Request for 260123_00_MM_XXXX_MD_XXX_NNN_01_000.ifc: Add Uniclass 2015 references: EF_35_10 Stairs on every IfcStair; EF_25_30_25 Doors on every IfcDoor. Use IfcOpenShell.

First a look at what the model holds.

```python
import ifcopenshell

model = ifcopenshell.open("260123_00_MM_XXXX_MD_XXX_NNN_01_000.ifc")
print(model.schema)
print("classifications:", [c.Name for c in model.by_type("IfcClassification")])
for ifc_class in ("IfcDoor", "IfcRoof", "IfcStair", "IfcWall", "IfcWindow"):
    print(ifc_class, len(model.by_type(ifc_class)))
```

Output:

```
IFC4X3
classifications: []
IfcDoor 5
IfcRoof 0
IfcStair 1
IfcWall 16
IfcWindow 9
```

```python
import ifcopenshell
import ifcopenshell.api.classification

model = ifcopenshell.open("260123_00_MM_XXXX_MD_XXX_NNN_01_000.ifc")

system = ifcopenshell.api.classification.add_classification(model, classification="Uniclass 2015")

codes = {
    "IfcStair": ("EF_35_10", "Stairs"),
    "IfcDoor": ("EF_25_30_25", "Doors"),
}
for ifc_class, (code, name) in codes.items():
    products = model.by_type(ifc_class)
    ifcopenshell.api.classification.add_reference(
        model, products=products, classification=system, identification=code, name=name
    )
    print(code, len(products))

model.write("260123_00_MM_XXXX_MD_XXX_NNN_01_000_rev.ifc")
```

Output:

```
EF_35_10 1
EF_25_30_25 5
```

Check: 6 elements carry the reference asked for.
